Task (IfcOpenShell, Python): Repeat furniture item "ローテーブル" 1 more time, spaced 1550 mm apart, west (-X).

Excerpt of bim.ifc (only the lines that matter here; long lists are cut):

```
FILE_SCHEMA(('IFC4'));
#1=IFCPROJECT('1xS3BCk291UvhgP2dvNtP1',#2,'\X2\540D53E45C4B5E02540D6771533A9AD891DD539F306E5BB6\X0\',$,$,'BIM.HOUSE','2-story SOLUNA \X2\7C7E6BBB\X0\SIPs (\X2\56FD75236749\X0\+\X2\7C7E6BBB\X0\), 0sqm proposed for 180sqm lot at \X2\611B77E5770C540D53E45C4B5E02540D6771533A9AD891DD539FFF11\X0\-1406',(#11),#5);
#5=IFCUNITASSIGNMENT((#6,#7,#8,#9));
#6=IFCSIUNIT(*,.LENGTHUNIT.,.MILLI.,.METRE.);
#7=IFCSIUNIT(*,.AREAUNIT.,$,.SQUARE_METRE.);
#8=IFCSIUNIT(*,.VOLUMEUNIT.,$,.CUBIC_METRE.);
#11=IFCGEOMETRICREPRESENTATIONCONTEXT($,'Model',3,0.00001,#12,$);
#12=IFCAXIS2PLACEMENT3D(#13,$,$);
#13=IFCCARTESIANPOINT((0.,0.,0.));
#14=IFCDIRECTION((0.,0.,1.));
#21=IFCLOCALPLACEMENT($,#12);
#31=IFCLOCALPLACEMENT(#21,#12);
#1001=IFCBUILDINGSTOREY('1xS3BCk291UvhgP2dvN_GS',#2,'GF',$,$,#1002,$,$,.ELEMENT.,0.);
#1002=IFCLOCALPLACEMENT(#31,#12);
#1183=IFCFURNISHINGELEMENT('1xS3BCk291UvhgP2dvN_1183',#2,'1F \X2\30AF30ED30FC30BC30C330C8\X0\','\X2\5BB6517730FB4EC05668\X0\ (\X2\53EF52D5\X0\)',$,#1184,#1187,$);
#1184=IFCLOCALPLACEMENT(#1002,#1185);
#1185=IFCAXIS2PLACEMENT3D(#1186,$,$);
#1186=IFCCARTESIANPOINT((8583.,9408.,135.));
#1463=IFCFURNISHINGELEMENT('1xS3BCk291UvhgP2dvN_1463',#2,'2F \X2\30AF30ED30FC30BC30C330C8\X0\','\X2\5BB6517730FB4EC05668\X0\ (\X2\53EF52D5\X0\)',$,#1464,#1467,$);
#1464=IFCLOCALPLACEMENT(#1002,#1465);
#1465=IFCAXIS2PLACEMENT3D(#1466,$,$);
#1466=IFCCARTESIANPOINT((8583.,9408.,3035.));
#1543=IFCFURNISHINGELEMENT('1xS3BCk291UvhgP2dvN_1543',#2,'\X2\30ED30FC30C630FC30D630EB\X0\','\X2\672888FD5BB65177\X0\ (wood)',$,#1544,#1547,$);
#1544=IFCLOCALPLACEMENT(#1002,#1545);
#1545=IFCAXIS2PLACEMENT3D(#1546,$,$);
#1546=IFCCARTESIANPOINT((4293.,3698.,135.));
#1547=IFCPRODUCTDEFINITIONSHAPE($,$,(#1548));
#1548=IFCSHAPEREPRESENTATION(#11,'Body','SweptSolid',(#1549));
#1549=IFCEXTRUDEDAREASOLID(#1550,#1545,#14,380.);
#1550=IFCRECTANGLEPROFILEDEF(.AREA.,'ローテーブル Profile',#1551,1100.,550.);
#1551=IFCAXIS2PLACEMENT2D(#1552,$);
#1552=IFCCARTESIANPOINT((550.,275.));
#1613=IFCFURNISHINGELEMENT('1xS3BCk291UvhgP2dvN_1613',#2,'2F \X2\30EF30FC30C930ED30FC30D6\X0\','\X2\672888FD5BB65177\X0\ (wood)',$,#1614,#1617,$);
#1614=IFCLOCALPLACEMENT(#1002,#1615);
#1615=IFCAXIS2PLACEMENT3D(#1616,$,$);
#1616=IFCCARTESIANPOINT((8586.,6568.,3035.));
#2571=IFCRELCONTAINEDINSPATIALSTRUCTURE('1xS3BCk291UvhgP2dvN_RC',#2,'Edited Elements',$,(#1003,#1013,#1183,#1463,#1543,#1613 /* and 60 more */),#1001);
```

```python
import numpy as np
import ifcopenshell
import ifcopenshell.api.geometry
import ifcopenshell.api.root
import ifcopenshell.util.element
import ifcopenshell.util.placement

model = ifcopenshell.open("bim.ifc")


def reuse_history(source, copy):
    """copy_class also copies each property set's owner history, people and application; keep the originals."""
    for rel in copy.IsDefinedBy:
        if rel.is_a("IfcRelDefinesByProperties") and (history := rel.RelatingPropertyDefinition.OwnerHistory):
            rel.RelatingPropertyDefinition.OwnerHistory = source.OwnerHistory
            ifcopenshell.util.element.remove_deep2(model, history)


source = model.by_id(1543)
base = ifcopenshell.util.placement.get_local_placement(source.ObjectPlacement)
step = np.array([-1.0, 0.0, 0.0]) * 1550.0

for i in range(1, 2):
    copy = ifcopenshell.api.root.copy_class(model, product=source)
    copy.Representation = ifcopenshell.util.element.copy_deep(
        model, source.Representation, exclude=["IfcGeometricRepresentationContext", "IfcRepresentationMap"]
    )
    reuse_history(source, copy)
    matrix = base.copy()
    matrix[:3, 3] += i * step
    print("added at", matrix[:3, 3].round(3) + 0.0)
    ifcopenshell.api.geometry.edit_object_placement(model, product=copy, matrix=matrix, is_si=False)

model.write("bim_updated.ifc")
```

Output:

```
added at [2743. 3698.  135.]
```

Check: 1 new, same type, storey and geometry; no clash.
